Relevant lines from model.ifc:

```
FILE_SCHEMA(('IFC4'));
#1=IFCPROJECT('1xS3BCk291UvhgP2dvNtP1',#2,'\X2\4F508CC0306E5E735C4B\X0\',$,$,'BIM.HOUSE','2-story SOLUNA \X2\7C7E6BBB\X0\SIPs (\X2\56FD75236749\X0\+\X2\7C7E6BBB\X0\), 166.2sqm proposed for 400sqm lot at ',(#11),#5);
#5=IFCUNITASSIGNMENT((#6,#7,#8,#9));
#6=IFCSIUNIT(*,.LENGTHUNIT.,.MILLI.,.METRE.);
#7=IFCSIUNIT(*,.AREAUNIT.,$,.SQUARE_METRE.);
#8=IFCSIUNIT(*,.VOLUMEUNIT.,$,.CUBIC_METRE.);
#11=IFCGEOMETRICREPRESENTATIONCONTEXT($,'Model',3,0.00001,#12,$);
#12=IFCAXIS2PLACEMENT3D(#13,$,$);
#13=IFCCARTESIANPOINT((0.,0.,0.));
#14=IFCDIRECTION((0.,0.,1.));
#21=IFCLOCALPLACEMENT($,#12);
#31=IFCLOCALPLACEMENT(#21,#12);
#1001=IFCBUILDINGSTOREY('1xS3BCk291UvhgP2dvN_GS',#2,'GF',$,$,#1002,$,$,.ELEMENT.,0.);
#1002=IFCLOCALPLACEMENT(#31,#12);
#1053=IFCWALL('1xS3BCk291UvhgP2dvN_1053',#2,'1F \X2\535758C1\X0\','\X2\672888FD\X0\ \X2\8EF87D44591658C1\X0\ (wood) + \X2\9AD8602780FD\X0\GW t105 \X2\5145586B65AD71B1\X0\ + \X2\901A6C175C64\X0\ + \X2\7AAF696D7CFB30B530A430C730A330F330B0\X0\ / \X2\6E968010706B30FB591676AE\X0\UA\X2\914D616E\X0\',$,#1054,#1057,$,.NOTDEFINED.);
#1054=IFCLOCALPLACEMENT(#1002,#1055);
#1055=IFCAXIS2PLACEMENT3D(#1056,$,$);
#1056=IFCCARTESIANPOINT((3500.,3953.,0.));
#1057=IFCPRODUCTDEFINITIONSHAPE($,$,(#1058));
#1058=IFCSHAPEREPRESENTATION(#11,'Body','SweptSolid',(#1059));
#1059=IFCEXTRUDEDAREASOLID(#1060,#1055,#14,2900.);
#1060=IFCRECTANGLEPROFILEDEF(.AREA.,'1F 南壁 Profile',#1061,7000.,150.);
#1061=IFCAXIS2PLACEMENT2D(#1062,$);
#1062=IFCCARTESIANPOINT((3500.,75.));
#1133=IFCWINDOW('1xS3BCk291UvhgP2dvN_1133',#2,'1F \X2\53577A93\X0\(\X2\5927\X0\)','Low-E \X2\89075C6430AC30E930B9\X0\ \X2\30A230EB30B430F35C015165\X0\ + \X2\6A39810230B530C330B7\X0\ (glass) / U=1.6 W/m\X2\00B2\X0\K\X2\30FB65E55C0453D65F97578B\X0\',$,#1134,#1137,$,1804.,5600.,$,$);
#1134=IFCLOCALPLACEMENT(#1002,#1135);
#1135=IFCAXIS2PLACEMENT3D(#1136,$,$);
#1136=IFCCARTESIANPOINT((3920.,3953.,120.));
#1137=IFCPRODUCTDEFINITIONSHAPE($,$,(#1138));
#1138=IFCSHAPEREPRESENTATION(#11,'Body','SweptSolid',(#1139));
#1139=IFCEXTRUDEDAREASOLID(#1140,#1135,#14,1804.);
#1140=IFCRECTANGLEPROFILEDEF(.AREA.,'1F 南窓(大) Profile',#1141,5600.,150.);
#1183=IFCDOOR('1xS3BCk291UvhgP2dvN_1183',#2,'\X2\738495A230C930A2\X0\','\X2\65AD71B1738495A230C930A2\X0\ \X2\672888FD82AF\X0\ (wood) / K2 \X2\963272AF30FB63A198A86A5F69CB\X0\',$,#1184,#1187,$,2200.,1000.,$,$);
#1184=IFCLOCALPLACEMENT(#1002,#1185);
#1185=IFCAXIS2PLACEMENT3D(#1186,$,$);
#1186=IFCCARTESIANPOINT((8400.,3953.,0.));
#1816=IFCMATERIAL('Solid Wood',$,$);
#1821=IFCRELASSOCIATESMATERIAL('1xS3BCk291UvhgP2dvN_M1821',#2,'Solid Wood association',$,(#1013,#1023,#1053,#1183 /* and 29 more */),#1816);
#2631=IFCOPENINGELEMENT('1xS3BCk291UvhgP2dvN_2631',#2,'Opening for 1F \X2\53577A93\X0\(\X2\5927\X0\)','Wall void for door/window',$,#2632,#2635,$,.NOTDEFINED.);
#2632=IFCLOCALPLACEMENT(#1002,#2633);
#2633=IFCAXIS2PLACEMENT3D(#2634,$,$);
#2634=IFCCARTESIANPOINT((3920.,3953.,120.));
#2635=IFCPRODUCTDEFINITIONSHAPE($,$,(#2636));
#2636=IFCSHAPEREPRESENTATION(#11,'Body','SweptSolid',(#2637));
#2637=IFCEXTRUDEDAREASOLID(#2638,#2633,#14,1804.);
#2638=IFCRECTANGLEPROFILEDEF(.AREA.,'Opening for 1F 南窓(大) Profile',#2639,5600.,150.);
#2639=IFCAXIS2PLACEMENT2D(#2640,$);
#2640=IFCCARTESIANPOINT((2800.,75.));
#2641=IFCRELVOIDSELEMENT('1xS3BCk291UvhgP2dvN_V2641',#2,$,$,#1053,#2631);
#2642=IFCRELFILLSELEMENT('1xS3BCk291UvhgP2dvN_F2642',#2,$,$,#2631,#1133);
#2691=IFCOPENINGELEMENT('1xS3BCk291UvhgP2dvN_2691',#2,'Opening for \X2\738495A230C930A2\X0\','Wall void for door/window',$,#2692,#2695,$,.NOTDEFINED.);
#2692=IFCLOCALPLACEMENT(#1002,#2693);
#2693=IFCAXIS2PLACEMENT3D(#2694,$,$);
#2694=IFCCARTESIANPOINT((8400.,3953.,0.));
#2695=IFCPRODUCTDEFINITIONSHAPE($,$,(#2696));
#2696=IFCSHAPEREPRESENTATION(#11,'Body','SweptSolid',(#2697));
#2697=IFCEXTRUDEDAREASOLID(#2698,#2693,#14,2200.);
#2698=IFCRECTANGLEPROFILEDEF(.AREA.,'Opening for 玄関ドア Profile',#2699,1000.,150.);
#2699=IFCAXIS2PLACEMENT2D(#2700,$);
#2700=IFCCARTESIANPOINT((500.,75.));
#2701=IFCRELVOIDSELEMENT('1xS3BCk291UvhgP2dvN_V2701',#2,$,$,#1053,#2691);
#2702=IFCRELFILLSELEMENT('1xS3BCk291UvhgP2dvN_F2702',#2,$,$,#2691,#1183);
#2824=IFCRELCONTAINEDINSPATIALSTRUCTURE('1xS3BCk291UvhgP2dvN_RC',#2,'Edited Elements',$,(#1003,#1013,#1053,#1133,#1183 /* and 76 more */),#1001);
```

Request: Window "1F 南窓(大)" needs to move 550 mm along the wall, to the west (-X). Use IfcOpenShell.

```python
import ifcopenshell
import ifcopenshell.api.geometry
import ifcopenshell.util.placement

model = ifcopenshell.open("model.ifc")

window = model.by_guid("1xS3BCk291UvhgP2dvN_1133")
opening = window.FillsVoids[0].RelatingOpeningElement
wall = opening.VoidsElements[0].RelatingBuildingElement

wall_matrix = ifcopenshell.util.placement.get_local_placement(wall.ObjectPlacement)
shift = wall_matrix[:3, 0] * -550.0
before = ifcopenshell.util.placement.get_local_placement(window.ObjectPlacement)[:3, 3].copy()

# The window is not placed relative to its opening, so move both.
for product in (opening, window):
    matrix = ifcopenshell.util.placement.get_local_placement(product.ObjectPlacement)
    matrix[:3, 3] += shift
    ifcopenshell.api.geometry.edit_object_placement(model, product=product, matrix=matrix, is_si=False)

after = ifcopenshell.util.placement.get_local_placement(window.ObjectPlacement)[:3, 3]
print("window moved by", (after - before).round(3) + 0.0)

model.write("model-out.ifc")
```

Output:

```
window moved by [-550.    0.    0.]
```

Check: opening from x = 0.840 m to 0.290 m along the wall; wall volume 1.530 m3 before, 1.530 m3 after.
